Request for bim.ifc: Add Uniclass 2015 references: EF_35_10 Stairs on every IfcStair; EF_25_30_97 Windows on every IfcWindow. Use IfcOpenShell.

First a look at what the model holds.

```python
import ifcopenshell

model = ifcopenshell.open("bim.ifc")
print(model.schema)
print("classifications:", [c.Name for c in model.by_type("IfcClassification")])
for ifc_class in ("IfcDoor", "IfcRoof", "IfcStair", "IfcWall", "IfcWindow"):
    print(ifc_class, len(model.by_type(ifc_class)))
```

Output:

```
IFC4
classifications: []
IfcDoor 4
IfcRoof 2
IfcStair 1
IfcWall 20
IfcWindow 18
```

```python
import ifcopenshell
import ifcopenshell.api.classification

model = ifcopenshell.open("bim.ifc")

system = ifcopenshell.api.classification.add_classification(model, classification="Uniclass 2015")

codes = {
    "IfcStair": ("EF_35_10", "Stairs"),
    "IfcWindow": ("EF_25_30_97", "Windows"),
}
for ifc_class, (code, name) in codes.items():
    products = model.by_type(ifc_class)
    ifcopenshell.api.classification.add_reference(
        model, products=products, classification=system, identification=code, name=name
    )
    print(code, len(products))

model.write("bim_v2.ifc")
```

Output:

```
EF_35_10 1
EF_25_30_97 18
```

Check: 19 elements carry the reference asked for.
